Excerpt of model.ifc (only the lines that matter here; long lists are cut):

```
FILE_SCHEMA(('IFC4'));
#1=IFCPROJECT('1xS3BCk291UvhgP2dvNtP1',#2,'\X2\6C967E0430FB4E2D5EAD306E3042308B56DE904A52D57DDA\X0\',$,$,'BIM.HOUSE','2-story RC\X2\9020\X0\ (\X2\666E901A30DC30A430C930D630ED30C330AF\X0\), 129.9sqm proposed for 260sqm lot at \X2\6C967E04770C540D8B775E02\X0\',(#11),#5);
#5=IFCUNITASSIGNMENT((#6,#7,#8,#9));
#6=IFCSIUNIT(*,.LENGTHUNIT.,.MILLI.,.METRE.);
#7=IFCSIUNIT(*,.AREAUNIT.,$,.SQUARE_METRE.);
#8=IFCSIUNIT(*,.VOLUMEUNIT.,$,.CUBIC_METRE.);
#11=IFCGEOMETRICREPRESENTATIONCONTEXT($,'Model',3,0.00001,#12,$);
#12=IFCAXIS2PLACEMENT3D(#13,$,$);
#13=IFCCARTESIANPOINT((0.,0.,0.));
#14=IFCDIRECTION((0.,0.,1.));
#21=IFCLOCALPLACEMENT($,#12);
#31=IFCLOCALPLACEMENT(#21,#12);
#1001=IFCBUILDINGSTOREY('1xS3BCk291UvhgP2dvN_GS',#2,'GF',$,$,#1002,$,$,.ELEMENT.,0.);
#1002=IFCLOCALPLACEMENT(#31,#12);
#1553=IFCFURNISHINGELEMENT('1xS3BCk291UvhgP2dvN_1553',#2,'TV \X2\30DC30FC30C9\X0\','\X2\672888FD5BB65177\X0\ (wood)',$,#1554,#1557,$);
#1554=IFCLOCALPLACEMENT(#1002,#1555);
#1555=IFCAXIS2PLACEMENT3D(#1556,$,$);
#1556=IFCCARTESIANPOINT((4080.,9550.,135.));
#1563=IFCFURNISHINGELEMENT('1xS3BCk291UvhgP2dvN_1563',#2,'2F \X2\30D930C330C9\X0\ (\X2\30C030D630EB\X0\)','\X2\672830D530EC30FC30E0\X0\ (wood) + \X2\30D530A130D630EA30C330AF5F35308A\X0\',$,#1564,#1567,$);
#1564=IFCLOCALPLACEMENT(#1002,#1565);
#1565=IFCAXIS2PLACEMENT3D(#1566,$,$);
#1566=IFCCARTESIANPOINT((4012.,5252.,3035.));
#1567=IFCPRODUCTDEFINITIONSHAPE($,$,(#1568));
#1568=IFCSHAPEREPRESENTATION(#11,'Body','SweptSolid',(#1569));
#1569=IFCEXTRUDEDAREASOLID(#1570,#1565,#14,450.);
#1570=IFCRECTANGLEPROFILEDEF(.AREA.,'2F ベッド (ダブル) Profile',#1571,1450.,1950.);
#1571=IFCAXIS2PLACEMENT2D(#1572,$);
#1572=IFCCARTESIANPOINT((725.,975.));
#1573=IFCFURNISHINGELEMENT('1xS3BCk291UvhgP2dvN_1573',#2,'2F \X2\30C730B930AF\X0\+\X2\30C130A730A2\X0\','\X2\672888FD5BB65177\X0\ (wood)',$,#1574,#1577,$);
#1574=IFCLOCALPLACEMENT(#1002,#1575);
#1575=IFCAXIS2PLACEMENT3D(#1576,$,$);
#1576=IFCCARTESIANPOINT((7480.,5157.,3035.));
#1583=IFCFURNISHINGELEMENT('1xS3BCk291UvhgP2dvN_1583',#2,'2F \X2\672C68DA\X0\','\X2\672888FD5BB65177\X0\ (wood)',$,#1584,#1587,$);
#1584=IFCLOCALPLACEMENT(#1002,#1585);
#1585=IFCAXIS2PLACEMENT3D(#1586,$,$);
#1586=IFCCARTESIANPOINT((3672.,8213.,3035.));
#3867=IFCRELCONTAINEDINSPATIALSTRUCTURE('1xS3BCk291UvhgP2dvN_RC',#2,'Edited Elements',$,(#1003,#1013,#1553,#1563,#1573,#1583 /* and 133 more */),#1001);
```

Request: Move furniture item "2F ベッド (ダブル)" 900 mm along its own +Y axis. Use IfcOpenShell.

```python
import ifcopenshell
import ifcopenshell.api.geometry
import ifcopenshell.util.placement

model = ifcopenshell.open("model.ifc")

item = model.by_guid("1xS3BCk291UvhgP2dvN_1563")
matrix = ifcopenshell.util.placement.get_local_placement(item.ObjectPlacement)
matrix[:3, 3] += matrix[:3, 1] * 900.0
ifcopenshell.api.geometry.edit_object_placement(model, product=item, matrix=matrix, is_si=False)

print(ifcopenshell.util.placement.get_local_placement(item.ObjectPlacement).round(3) + 0.0)

model.write("model_rev.ifc")
```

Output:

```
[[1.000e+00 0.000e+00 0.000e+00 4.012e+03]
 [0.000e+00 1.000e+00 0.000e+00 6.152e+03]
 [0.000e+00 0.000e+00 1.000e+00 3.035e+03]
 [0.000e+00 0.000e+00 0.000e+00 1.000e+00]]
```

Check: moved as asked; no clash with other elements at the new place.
